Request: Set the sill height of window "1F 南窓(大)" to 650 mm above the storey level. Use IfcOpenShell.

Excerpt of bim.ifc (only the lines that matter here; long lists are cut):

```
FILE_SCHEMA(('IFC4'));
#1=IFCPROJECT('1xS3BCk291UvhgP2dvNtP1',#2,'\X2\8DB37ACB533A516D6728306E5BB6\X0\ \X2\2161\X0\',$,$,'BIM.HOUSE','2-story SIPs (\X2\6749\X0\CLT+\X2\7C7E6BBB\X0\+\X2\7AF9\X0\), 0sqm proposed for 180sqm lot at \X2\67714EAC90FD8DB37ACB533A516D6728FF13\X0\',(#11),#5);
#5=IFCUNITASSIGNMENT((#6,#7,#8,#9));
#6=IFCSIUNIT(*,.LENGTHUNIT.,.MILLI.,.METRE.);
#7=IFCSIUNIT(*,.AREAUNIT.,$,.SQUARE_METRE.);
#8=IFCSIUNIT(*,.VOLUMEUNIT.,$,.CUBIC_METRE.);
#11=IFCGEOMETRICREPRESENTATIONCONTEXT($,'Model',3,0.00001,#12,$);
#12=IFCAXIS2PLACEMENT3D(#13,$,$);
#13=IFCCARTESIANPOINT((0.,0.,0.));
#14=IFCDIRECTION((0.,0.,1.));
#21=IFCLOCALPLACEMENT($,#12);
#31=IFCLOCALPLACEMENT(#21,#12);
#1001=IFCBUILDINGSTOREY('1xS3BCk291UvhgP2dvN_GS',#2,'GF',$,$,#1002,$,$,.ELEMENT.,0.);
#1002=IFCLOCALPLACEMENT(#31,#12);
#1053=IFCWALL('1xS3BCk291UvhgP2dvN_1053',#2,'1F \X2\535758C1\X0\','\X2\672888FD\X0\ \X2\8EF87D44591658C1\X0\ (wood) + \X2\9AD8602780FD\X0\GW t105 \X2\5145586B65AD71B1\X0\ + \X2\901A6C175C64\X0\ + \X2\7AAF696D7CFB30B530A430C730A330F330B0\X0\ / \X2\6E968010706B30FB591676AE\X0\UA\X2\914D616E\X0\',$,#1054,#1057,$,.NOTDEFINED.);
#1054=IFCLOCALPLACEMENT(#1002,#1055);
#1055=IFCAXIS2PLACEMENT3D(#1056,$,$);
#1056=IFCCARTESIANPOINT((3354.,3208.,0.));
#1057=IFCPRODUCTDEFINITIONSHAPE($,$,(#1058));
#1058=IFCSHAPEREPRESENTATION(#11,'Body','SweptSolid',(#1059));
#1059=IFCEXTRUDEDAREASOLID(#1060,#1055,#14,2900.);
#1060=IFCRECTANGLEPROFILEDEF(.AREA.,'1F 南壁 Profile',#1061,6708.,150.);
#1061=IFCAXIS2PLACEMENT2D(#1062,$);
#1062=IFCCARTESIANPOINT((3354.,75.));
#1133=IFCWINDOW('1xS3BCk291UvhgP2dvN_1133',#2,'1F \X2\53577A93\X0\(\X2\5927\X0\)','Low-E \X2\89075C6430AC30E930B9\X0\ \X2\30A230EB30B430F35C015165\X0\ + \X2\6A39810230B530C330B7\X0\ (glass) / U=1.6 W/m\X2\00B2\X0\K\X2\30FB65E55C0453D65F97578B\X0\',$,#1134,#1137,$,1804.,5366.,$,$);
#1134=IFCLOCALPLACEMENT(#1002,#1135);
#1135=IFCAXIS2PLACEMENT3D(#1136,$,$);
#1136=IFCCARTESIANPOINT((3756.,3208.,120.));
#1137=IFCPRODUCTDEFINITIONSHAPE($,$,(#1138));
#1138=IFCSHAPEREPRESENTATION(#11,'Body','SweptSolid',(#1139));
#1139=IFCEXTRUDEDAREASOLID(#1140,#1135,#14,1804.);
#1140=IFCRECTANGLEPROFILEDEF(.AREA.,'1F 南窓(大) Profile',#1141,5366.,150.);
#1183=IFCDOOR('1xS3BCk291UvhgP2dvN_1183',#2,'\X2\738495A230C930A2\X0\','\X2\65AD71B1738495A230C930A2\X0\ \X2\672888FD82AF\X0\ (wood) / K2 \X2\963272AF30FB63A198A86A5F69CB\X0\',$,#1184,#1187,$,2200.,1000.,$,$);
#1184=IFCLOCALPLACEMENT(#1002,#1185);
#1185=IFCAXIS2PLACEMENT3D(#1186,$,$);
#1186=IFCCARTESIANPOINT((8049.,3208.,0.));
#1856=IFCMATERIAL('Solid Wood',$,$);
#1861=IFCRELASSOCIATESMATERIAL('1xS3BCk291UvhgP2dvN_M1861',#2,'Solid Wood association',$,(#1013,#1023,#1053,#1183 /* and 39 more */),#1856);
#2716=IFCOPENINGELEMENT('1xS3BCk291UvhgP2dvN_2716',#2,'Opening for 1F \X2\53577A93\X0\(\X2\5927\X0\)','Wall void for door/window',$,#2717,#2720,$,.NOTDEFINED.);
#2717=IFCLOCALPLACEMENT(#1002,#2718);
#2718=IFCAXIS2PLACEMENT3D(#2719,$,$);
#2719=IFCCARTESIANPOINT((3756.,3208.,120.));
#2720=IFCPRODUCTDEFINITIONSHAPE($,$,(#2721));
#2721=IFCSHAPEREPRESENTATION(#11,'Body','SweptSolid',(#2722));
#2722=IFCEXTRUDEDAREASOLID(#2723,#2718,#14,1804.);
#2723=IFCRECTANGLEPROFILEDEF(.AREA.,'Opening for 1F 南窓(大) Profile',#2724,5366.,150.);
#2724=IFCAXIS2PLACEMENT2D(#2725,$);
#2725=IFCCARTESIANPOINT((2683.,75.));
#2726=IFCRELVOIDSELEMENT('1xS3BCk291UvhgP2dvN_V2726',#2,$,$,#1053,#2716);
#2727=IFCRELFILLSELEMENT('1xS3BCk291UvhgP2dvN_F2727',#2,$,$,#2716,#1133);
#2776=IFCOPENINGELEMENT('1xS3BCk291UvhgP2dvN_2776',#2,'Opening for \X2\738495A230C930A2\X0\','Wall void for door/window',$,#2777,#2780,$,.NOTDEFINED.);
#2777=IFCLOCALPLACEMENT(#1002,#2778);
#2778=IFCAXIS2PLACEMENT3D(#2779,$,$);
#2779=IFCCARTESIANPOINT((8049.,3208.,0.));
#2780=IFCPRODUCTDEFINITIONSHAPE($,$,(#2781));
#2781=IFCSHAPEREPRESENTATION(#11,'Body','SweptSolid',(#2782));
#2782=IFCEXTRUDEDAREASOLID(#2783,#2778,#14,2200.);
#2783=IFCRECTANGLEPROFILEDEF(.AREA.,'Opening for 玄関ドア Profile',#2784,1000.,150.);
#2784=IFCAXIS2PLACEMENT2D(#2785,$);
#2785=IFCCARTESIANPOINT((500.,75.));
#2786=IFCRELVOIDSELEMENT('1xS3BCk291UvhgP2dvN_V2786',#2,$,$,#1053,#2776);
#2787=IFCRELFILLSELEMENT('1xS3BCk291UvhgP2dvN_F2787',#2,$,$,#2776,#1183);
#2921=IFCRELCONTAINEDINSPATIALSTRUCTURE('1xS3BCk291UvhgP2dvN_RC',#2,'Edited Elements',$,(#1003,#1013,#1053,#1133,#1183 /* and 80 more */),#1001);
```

```python
import numpy as np
import ifcopenshell
import ifcopenshell.api.geometry
import ifcopenshell.geom
import ifcopenshell.util.element
import ifcopenshell.util.placement
import ifcopenshell.util.shape
import ifcopenshell.util.unit

model = ifcopenshell.open("bim.ifc")
unit_scale = ifcopenshell.util.unit.calculate_unit_scale(model)

window = model.by_guid("1xS3BCk291UvhgP2dvN_1133")
opening = window.FillsVoids[0].RelatingOpeningElement
storey = ifcopenshell.util.element.get_container(window, ifc_class="IfcBuildingStorey")
level = ifcopenshell.util.placement.get_local_placement(storey.ObjectPlacement)[2, 3]

# The opening's origin need not be at the sill, so measure its lowest point.
shape = ifcopenshell.geom.create_shape(ifcopenshell.geom.settings(), opening)
bottom = ifcopenshell.util.shape.get_shape_bottom_elevation(shape, shape.geometry) / unit_scale
dz = level + 650.0 - bottom

shift = np.array([0.0, 0.0, dz])
# The window is not placed relative to its opening, so move both.
for product in (opening, window):
    matrix = ifcopenshell.util.placement.get_local_placement(product.ObjectPlacement)
    matrix[:3, 3] += shift
    ifcopenshell.api.geometry.edit_object_placement(model, product=product, matrix=matrix, is_si=False)

print(f"moved by {dz * unit_scale:+.3f} m")

model.write("bim_rev.ifc")
```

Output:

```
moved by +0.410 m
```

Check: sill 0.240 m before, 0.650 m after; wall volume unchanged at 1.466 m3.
